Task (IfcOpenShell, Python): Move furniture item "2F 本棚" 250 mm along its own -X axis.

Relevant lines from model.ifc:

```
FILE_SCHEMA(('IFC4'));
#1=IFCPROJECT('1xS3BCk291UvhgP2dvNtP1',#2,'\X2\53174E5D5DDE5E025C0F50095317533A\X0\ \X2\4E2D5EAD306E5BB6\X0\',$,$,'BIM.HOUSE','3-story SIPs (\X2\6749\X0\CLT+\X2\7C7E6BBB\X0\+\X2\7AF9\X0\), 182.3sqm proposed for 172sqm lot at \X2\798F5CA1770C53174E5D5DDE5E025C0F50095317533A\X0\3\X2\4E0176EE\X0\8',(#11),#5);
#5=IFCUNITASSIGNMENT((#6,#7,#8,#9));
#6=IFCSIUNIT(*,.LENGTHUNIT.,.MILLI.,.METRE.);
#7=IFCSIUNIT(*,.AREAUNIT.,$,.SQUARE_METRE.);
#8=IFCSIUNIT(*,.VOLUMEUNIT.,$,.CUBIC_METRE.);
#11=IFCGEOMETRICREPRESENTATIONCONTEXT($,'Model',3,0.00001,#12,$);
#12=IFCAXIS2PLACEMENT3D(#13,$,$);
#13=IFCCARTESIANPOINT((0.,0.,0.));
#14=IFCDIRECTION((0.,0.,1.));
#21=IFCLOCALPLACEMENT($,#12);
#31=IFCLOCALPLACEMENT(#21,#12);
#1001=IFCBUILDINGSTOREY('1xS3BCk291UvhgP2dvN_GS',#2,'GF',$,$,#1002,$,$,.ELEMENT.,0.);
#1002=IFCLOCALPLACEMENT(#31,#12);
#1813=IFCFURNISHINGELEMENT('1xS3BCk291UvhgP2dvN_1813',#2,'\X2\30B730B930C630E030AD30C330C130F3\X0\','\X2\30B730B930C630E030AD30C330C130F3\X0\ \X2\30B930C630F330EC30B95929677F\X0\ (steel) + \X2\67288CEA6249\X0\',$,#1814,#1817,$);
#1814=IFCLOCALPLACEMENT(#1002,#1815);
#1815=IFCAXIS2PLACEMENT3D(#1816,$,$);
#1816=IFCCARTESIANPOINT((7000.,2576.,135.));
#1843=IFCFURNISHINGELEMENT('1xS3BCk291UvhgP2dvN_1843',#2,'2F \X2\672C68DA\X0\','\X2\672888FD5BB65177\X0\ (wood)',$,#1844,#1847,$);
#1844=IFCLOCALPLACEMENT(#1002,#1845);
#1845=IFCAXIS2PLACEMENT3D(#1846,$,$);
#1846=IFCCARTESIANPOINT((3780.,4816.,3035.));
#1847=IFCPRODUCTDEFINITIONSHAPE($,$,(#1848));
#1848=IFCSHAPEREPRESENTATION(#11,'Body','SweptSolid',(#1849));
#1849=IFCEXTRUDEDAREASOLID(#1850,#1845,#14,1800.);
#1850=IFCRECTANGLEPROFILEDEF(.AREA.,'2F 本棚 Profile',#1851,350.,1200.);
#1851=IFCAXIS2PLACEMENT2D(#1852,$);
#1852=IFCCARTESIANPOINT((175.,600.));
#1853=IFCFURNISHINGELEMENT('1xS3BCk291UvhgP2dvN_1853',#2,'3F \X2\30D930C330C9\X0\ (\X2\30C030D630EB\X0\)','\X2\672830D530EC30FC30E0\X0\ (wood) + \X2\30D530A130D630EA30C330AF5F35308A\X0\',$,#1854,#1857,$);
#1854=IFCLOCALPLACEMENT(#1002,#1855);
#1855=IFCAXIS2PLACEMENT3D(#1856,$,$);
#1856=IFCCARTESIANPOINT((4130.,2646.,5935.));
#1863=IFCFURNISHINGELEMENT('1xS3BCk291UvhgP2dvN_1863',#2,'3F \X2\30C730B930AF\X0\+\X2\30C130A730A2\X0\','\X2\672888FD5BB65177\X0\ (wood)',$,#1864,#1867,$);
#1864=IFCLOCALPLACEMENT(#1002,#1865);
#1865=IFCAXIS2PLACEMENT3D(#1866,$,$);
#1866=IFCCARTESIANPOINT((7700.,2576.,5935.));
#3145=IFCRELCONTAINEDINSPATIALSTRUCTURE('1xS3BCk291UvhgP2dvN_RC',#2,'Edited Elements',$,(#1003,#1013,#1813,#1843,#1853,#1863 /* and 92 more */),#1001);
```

```python
import ifcopenshell
import ifcopenshell.api.geometry
import ifcopenshell.util.placement
import ifcopenshell.util.unit

model = ifcopenshell.open("model.ifc")
unit_scale = ifcopenshell.util.unit.calculate_unit_scale(model)

item = model.by_guid("1xS3BCk291UvhgP2dvN_1843")
matrix = ifcopenshell.util.placement.get_local_placement(item.ObjectPlacement)
matrix[:3, 3] -= matrix[:3, 0] * 0.25 / unit_scale
ifcopenshell.api.geometry.edit_object_placement(model, product=item, matrix=matrix, is_si=False)

print(ifcopenshell.util.placement.get_local_placement(item.ObjectPlacement).round(3) + 0.0)

model.write("model_rev.ifc")
```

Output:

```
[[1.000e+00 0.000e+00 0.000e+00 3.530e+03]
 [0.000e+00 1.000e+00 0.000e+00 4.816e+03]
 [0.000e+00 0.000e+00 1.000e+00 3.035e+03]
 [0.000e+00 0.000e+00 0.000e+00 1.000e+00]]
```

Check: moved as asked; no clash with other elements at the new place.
